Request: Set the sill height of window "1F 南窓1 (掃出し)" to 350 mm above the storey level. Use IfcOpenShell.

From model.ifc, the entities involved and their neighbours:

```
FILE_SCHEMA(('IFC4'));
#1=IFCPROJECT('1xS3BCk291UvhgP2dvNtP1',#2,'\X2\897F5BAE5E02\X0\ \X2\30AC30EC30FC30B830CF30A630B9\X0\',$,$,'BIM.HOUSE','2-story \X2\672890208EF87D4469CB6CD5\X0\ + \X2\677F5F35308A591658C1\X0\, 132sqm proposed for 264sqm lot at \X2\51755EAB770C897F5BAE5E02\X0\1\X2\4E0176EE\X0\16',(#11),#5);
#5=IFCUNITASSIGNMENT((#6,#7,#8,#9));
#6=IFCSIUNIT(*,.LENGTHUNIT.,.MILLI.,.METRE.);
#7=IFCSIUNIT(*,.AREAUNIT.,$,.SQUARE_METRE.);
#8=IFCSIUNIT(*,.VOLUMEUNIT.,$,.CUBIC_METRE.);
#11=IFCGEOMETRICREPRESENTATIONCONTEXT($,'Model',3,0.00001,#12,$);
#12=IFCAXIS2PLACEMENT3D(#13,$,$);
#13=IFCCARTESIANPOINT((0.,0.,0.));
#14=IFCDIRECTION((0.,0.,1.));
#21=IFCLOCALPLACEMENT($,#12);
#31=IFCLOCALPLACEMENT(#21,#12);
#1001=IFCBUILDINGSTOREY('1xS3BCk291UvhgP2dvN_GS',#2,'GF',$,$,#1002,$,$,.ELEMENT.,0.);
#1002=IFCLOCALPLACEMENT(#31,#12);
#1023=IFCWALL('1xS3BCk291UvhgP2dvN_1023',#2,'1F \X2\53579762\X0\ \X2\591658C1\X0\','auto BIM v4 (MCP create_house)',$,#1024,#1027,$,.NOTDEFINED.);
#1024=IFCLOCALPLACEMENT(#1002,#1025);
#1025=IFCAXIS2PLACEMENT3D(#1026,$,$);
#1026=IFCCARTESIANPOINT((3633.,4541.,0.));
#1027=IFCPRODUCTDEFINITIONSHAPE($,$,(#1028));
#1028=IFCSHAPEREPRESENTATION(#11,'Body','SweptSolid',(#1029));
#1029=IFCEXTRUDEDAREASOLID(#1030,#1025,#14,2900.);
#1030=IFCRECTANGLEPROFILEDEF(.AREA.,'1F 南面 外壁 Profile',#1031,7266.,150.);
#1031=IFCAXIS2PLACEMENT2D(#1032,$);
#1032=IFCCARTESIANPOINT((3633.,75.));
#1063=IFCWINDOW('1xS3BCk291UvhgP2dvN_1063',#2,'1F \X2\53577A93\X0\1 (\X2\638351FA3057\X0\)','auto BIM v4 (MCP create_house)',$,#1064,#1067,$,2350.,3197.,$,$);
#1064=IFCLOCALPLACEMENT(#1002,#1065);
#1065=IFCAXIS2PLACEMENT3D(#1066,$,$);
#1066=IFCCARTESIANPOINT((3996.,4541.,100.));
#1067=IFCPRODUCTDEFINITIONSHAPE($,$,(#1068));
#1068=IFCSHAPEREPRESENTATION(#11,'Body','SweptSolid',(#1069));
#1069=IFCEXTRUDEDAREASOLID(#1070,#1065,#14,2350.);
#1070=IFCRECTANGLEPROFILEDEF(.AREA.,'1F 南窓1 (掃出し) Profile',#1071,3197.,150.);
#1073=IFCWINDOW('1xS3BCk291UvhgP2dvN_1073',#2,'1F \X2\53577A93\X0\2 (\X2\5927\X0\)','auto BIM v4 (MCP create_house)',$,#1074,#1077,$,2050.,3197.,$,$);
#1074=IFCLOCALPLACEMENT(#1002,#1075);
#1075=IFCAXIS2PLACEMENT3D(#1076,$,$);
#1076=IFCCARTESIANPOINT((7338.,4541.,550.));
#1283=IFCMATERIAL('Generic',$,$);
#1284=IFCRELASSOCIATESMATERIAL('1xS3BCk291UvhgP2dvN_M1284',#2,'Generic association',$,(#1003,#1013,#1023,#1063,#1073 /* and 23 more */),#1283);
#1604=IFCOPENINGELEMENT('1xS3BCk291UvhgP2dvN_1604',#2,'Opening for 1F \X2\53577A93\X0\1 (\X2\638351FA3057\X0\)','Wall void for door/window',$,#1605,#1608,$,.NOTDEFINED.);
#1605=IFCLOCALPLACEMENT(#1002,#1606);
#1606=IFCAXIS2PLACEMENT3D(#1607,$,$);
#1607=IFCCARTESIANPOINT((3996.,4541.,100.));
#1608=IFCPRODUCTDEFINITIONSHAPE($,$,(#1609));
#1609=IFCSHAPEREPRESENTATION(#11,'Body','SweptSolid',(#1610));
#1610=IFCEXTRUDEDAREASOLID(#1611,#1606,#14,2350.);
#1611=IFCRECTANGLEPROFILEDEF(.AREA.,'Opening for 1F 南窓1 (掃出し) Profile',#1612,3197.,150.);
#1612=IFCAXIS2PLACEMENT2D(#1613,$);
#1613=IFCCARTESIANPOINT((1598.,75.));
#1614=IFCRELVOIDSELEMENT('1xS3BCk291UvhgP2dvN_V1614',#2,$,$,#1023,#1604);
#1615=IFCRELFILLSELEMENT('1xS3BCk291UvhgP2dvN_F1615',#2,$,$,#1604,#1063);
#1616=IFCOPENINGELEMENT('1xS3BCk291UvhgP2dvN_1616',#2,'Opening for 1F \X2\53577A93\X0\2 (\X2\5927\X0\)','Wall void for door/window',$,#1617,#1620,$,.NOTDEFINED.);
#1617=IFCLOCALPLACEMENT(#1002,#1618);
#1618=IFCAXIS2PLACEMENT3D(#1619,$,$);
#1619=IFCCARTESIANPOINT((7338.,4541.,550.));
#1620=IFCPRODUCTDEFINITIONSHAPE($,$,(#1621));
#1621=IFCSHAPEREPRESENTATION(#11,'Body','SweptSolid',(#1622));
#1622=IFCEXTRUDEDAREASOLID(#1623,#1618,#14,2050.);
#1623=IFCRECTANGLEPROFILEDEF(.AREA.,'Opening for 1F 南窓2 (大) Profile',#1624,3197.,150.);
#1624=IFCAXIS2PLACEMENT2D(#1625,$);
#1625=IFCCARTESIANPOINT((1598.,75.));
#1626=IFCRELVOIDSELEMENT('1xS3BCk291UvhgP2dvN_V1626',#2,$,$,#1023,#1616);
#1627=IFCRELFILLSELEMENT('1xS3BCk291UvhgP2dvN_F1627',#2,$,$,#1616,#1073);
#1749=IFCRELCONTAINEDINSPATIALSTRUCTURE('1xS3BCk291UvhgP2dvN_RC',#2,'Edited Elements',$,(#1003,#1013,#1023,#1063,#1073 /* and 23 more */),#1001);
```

```python
import numpy as np
import ifcopenshell
import ifcopenshell.api.geometry
import ifcopenshell.geom
import ifcopenshell.util.element
import ifcopenshell.util.placement
import ifcopenshell.util.shape
import ifcopenshell.util.unit

model = ifcopenshell.open("model.ifc")
unit_scale = ifcopenshell.util.unit.calculate_unit_scale(model)

window = model.by_guid("1xS3BCk291UvhgP2dvN_1063")
opening = window.FillsVoids[0].RelatingOpeningElement
storey = ifcopenshell.util.element.get_container(window, ifc_class="IfcBuildingStorey")
level = ifcopenshell.util.placement.get_local_placement(storey.ObjectPlacement)[2, 3]

# The opening's origin need not be at the sill, so measure its lowest point.
shape = ifcopenshell.geom.create_shape(ifcopenshell.geom.settings(), opening)
bottom = ifcopenshell.util.shape.get_shape_bottom_elevation(shape, shape.geometry) / unit_scale
dz = level + 350.0 - bottom

shift = np.array([0.0, 0.0, dz])
# The window is not placed relative to its opening, so move both.
for product in (opening, window):
    matrix = ifcopenshell.util.placement.get_local_placement(product.ObjectPlacement)
    matrix[:3, 3] += shift
    ifcopenshell.api.geometry.edit_object_placement(model, product=product, matrix=matrix, is_si=False)

print(f"moved by {dz * unit_scale:+.3f} m")

model.write("model_updated.ifc")
```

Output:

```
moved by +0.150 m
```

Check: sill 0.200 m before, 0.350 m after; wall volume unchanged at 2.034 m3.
